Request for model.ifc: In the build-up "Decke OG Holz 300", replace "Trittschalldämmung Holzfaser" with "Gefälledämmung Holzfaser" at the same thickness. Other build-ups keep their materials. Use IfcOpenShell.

First a look at what the model holds.

```python
import ifcopenshell
import ifcopenshell.util.element

model = ifcopenshell.open("model.ifc")
print(model.schema)
for layer_set in model.by_type("IfcMaterialLayerSet"):
    if layer_set.LayerSetName == "Decke OG Holz 300":
        for layer in layer_set.MaterialLayers:
            print(layer.id(), layer.Material and layer.Material.Name, layer.LayerThickness, sep=" | ")
        print(len(ifcopenshell.util.element.get_elements_by_material(model, layer_set)), "elements and types use it")
print(sorted(m.Name for m in model.by_type("IfcMaterial") if m.Name)[:60])
```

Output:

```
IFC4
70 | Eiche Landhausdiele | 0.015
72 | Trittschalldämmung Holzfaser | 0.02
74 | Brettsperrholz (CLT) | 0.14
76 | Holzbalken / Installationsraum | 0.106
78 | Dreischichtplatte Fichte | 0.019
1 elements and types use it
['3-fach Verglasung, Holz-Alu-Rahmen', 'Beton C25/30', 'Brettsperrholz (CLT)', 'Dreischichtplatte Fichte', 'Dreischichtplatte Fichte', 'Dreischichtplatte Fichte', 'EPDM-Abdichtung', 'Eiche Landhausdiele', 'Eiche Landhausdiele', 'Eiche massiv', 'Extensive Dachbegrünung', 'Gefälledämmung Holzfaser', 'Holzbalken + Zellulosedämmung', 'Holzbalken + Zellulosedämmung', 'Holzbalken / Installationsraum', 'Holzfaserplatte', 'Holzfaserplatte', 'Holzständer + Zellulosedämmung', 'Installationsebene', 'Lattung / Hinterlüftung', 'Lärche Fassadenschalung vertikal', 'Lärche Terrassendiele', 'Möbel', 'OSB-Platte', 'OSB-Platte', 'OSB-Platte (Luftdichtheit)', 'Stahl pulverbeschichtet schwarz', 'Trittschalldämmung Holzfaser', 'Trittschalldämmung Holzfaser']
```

```python
import ifcopenshell
import ifcopenshell.api.material

model = ifcopenshell.open("model.ifc")

layer_set = next(s for s in model.by_type("IfcMaterialLayerSet") if s.LayerSetName == "Decke OG Holz 300")
layer = next(l for l in layer_set.MaterialLayers if l.Material and l.Material.Name == "Trittschalldämmung Holzfaser")
material = next(m for m in model.by_type("IfcMaterial") if m.Name == "Gefälledämmung Holzfaser")

# Point this one layer at the other material; renaming the old one would change it everywhere.
ifcopenshell.api.material.edit_layer(model, layer=layer, attributes={"Name": material.Name}, material=material)

print([l.Material.Name if l.Material else None for l in layer_set.MaterialLayers])

model.write("model_rev.ifc")
```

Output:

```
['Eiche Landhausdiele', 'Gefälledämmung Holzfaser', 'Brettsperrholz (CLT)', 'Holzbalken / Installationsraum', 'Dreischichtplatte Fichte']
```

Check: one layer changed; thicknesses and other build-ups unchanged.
